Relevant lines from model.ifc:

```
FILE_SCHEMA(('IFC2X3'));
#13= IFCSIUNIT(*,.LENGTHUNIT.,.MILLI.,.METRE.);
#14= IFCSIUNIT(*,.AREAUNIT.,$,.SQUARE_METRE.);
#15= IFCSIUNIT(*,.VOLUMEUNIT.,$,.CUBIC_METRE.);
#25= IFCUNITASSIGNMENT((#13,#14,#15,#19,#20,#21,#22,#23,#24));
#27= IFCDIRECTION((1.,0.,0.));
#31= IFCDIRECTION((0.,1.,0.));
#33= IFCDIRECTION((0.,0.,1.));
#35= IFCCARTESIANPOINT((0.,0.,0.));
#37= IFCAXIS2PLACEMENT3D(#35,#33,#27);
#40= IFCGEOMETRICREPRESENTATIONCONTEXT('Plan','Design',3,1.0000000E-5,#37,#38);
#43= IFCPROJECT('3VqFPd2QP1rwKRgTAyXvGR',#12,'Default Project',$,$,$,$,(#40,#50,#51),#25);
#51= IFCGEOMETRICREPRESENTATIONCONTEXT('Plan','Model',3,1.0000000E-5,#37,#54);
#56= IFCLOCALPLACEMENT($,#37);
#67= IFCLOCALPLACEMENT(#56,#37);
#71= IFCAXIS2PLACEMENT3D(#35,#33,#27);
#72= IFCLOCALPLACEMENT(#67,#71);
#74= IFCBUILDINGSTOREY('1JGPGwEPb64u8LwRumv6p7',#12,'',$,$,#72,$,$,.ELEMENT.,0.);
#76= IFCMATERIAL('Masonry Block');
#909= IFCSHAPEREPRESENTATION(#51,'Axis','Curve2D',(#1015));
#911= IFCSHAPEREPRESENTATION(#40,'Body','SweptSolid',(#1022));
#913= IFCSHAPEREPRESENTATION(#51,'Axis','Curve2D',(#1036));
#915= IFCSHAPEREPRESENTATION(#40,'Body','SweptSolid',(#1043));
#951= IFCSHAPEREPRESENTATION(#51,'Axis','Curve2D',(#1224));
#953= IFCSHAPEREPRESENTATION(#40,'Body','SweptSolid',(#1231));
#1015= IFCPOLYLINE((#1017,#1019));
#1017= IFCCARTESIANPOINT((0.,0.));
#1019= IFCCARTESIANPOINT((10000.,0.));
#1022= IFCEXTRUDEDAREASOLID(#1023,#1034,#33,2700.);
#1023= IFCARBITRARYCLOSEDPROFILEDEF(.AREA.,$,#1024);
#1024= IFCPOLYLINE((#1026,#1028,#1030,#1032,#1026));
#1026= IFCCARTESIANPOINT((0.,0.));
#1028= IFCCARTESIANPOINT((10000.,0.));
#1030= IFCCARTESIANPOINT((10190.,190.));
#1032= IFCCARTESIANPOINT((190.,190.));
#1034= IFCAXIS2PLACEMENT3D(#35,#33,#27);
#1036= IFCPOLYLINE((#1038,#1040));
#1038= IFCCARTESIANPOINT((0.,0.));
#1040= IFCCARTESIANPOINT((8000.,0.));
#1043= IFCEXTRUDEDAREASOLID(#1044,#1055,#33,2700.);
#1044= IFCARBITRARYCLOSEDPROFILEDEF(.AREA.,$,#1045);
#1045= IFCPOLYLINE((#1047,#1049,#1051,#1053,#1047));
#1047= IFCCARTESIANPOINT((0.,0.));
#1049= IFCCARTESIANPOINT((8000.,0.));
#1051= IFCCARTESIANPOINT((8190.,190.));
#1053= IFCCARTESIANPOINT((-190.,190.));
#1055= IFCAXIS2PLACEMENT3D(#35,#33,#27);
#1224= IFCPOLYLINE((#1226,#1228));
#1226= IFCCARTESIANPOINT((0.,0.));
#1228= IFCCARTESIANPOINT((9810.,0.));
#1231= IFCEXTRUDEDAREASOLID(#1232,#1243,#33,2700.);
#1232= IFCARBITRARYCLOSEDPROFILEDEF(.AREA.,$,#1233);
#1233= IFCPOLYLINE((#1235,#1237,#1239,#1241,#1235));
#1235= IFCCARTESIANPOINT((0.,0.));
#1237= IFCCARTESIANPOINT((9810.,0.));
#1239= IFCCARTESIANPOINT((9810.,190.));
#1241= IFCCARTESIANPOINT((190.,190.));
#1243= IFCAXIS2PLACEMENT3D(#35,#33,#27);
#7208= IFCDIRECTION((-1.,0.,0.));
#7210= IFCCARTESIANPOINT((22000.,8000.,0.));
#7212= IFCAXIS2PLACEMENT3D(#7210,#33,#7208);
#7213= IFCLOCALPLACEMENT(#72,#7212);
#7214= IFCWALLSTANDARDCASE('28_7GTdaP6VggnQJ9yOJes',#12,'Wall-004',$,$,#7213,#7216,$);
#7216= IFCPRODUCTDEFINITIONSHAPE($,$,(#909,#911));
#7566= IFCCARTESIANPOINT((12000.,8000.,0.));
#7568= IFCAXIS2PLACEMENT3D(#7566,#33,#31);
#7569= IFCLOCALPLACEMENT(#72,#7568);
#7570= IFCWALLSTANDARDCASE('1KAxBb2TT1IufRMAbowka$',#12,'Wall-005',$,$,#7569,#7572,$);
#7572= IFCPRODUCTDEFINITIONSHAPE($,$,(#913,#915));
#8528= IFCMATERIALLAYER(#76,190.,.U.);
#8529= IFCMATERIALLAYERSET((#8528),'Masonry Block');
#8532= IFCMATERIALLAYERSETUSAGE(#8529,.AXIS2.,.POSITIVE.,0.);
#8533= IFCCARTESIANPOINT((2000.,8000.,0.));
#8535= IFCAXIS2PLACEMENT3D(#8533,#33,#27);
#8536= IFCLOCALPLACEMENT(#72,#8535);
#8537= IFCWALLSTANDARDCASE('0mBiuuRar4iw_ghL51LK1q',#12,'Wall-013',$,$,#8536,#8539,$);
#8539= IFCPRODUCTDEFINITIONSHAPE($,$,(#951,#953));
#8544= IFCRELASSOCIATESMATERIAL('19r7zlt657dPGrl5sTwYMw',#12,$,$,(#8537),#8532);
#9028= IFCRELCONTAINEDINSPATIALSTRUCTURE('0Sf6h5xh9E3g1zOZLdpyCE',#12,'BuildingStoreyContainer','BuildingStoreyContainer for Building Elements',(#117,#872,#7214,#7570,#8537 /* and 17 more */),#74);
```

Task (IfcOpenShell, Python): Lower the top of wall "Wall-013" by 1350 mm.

```python
import ifcopenshell
import ifcopenshell.geom
import ifcopenshell.util.shape

model = ifcopenshell.open("model.ifc")
settings = ifcopenshell.geom.settings()


def volume(element):
    """Net volume in cubic metres, openings subtracted."""
    shape = ifcopenshell.geom.create_shape(settings, element)
    return ifcopenshell.util.shape.get_volume(shape.geometry)


wall = model.by_guid("0mBiuuRar4iw_ghL51LK1q")
before = volume(wall)

body = next(r for r in wall.Representation.Representations if r.RepresentationIdentifier == "Body")
solid = body.Items[0]
old_height = solid.Depth
solid.Depth -= 1350.0
after = volume(wall)

print(f"height {old_height:g} -> {solid.Depth:g}, volume {before:.3f} -> {after:.3f} m3")

model.write("model-out.ifc")
```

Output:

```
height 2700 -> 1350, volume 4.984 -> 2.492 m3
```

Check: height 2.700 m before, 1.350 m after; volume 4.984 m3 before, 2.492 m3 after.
